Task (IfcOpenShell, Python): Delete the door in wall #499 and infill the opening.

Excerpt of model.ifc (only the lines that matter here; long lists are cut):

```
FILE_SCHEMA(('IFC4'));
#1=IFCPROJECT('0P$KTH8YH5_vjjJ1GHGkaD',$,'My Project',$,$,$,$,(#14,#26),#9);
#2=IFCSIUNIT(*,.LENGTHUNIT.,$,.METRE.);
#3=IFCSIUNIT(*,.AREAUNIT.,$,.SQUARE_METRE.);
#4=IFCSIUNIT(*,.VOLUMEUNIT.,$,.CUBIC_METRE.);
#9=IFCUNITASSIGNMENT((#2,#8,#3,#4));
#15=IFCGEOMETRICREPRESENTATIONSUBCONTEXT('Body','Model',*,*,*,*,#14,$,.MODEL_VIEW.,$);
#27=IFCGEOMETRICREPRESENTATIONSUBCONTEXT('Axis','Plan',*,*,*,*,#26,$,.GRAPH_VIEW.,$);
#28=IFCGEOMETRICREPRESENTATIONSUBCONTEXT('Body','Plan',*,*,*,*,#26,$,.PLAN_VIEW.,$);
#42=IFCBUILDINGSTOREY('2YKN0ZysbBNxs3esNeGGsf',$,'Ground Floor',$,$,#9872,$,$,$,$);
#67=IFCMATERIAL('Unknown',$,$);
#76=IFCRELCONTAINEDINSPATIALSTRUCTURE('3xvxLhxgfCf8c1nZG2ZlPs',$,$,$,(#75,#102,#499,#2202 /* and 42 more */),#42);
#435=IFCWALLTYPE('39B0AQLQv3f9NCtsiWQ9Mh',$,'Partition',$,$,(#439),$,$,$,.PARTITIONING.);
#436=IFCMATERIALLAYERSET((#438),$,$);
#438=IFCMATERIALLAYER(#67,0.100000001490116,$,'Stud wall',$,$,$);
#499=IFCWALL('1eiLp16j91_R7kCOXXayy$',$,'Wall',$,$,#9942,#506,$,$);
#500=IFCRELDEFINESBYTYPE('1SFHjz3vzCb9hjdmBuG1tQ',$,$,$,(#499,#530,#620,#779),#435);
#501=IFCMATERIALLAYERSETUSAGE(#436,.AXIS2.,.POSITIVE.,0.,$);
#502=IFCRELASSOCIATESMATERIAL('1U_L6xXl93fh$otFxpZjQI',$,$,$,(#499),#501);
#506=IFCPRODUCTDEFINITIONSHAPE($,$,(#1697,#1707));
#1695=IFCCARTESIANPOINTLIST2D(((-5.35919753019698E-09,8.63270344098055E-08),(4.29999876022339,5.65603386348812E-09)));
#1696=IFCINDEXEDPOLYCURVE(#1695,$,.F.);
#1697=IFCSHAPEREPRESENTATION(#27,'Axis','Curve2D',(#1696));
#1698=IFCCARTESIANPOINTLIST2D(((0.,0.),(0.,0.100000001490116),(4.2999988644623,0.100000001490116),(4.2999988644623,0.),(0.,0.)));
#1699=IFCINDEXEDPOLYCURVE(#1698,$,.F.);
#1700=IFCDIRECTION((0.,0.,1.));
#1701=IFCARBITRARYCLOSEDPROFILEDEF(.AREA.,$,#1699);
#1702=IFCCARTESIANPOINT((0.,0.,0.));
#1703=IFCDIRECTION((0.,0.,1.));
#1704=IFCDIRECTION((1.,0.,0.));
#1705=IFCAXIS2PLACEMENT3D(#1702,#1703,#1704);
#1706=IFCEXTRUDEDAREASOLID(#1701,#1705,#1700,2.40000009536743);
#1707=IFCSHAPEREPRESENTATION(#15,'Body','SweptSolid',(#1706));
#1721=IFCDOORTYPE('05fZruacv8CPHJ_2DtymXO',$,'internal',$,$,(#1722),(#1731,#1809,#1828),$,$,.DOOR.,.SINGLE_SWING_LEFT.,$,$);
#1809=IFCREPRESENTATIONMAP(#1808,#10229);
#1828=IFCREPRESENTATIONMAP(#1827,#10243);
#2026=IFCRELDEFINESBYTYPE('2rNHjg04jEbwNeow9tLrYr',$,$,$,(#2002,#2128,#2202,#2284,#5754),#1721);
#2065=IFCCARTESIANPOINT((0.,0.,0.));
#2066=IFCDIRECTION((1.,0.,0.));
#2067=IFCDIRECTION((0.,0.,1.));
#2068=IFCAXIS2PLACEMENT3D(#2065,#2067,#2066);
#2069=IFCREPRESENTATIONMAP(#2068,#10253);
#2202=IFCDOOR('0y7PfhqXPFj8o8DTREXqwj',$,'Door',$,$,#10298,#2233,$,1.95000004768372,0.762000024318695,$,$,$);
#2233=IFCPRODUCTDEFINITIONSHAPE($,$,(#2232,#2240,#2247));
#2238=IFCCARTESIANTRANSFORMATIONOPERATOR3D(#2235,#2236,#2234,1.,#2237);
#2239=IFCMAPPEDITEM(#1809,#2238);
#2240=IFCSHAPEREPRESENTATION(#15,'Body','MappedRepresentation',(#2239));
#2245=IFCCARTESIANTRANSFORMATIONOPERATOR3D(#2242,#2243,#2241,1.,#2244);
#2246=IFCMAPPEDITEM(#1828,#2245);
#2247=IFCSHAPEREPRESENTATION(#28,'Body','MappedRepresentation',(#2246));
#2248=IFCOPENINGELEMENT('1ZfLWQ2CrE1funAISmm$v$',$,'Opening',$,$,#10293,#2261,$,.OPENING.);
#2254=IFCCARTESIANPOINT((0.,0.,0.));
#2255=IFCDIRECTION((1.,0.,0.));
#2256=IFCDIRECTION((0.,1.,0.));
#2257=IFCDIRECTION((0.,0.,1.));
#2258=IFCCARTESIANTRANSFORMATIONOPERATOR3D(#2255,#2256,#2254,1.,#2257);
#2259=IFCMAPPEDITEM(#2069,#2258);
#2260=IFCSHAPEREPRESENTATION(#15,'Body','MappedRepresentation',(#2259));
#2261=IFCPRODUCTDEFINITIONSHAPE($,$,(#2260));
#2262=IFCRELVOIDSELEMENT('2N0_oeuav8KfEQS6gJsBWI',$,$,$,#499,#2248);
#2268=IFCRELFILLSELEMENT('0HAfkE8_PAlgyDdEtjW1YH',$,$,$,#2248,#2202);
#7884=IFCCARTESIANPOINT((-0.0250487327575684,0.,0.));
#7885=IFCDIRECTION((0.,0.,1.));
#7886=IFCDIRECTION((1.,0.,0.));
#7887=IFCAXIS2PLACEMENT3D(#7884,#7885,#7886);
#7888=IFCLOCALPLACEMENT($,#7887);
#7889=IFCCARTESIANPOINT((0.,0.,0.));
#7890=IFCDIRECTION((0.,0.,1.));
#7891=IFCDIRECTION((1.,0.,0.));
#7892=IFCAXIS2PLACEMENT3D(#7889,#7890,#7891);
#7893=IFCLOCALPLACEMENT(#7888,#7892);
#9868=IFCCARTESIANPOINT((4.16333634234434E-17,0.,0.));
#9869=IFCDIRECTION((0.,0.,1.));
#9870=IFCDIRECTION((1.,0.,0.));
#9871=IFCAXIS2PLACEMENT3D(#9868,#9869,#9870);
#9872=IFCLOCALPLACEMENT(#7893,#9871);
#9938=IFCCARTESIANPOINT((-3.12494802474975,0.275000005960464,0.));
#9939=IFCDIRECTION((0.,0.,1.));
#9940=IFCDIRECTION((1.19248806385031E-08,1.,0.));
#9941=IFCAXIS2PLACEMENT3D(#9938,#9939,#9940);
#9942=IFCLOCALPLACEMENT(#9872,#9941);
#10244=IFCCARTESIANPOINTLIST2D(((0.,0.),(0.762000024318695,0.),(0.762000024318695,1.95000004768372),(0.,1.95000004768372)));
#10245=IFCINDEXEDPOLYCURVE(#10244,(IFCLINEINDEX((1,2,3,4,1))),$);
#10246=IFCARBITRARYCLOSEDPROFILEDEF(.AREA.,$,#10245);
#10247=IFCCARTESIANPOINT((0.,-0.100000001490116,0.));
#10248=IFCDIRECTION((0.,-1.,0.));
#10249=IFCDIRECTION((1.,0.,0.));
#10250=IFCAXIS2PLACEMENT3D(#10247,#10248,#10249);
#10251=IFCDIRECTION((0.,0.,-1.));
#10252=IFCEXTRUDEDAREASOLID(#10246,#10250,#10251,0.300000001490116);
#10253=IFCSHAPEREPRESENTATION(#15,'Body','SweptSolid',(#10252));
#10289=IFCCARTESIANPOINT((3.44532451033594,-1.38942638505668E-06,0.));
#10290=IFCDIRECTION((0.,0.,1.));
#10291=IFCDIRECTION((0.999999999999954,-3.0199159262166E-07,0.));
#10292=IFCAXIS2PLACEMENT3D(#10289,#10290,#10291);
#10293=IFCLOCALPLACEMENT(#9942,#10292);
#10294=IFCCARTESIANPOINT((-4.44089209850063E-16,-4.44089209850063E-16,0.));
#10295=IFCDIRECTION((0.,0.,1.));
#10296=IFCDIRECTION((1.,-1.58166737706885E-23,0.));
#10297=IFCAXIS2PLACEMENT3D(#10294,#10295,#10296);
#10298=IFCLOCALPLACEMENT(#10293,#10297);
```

```python
import ifcopenshell
import ifcopenshell.api.feature
import ifcopenshell.api.root
import ifcopenshell.geom
import ifcopenshell.util.shape

model = ifcopenshell.open("model.ifc")
settings = ifcopenshell.geom.settings()


def volume(element):
    """Net volume in cubic metres, openings subtracted."""
    shape = ifcopenshell.geom.create_shape(settings, element)
    return ifcopenshell.util.shape.get_volume(shape.geometry)


door = model.by_id(2202)
opening = door.FillsVoids[0].RelatingOpeningElement
wall = opening.VoidsElements[0].RelatingBuildingElement
before = volume(wall)

ifcopenshell.api.root.remove_product(model, product=door)
ifcopenshell.api.feature.remove_feature(model, feature=opening)

after = volume(wall)

print(f"wall volume {before:.3f} -> {after:.3f} m3")

model.write("model_updated.ifc")
```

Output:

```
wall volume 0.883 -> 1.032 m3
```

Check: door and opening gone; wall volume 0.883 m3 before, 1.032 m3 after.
